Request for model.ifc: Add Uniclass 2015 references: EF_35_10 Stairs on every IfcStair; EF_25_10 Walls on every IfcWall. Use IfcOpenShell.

First a look at what the model holds.

```python
import ifcopenshell

model = ifcopenshell.open("model.ifc")
print(model.schema)
print("classifications:", [c.Name for c in model.by_type("IfcClassification")])
for ifc_class in ("IfcDoor", "IfcRoof", "IfcStair", "IfcWall", "IfcWindow"):
    print(ifc_class, len(model.by_type(ifc_class)))
```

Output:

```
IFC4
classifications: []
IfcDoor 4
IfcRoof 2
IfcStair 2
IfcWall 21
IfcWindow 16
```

```python
import ifcopenshell
import ifcopenshell.api.classification

model = ifcopenshell.open("model.ifc")

system = ifcopenshell.api.classification.add_classification(model, classification="Uniclass 2015")

codes = {
    "IfcStair": ("EF_35_10", "Stairs"),
    "IfcWall": ("EF_25_10", "Walls"),
}
for ifc_class, (code, name) in codes.items():
    products = model.by_type(ifc_class)
    ifcopenshell.api.classification.add_reference(
        model, products=products, classification=system, identification=code, name=name
    )
    print(code, len(products))

model.write("model_updated.ifc")
```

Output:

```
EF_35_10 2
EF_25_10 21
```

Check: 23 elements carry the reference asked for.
